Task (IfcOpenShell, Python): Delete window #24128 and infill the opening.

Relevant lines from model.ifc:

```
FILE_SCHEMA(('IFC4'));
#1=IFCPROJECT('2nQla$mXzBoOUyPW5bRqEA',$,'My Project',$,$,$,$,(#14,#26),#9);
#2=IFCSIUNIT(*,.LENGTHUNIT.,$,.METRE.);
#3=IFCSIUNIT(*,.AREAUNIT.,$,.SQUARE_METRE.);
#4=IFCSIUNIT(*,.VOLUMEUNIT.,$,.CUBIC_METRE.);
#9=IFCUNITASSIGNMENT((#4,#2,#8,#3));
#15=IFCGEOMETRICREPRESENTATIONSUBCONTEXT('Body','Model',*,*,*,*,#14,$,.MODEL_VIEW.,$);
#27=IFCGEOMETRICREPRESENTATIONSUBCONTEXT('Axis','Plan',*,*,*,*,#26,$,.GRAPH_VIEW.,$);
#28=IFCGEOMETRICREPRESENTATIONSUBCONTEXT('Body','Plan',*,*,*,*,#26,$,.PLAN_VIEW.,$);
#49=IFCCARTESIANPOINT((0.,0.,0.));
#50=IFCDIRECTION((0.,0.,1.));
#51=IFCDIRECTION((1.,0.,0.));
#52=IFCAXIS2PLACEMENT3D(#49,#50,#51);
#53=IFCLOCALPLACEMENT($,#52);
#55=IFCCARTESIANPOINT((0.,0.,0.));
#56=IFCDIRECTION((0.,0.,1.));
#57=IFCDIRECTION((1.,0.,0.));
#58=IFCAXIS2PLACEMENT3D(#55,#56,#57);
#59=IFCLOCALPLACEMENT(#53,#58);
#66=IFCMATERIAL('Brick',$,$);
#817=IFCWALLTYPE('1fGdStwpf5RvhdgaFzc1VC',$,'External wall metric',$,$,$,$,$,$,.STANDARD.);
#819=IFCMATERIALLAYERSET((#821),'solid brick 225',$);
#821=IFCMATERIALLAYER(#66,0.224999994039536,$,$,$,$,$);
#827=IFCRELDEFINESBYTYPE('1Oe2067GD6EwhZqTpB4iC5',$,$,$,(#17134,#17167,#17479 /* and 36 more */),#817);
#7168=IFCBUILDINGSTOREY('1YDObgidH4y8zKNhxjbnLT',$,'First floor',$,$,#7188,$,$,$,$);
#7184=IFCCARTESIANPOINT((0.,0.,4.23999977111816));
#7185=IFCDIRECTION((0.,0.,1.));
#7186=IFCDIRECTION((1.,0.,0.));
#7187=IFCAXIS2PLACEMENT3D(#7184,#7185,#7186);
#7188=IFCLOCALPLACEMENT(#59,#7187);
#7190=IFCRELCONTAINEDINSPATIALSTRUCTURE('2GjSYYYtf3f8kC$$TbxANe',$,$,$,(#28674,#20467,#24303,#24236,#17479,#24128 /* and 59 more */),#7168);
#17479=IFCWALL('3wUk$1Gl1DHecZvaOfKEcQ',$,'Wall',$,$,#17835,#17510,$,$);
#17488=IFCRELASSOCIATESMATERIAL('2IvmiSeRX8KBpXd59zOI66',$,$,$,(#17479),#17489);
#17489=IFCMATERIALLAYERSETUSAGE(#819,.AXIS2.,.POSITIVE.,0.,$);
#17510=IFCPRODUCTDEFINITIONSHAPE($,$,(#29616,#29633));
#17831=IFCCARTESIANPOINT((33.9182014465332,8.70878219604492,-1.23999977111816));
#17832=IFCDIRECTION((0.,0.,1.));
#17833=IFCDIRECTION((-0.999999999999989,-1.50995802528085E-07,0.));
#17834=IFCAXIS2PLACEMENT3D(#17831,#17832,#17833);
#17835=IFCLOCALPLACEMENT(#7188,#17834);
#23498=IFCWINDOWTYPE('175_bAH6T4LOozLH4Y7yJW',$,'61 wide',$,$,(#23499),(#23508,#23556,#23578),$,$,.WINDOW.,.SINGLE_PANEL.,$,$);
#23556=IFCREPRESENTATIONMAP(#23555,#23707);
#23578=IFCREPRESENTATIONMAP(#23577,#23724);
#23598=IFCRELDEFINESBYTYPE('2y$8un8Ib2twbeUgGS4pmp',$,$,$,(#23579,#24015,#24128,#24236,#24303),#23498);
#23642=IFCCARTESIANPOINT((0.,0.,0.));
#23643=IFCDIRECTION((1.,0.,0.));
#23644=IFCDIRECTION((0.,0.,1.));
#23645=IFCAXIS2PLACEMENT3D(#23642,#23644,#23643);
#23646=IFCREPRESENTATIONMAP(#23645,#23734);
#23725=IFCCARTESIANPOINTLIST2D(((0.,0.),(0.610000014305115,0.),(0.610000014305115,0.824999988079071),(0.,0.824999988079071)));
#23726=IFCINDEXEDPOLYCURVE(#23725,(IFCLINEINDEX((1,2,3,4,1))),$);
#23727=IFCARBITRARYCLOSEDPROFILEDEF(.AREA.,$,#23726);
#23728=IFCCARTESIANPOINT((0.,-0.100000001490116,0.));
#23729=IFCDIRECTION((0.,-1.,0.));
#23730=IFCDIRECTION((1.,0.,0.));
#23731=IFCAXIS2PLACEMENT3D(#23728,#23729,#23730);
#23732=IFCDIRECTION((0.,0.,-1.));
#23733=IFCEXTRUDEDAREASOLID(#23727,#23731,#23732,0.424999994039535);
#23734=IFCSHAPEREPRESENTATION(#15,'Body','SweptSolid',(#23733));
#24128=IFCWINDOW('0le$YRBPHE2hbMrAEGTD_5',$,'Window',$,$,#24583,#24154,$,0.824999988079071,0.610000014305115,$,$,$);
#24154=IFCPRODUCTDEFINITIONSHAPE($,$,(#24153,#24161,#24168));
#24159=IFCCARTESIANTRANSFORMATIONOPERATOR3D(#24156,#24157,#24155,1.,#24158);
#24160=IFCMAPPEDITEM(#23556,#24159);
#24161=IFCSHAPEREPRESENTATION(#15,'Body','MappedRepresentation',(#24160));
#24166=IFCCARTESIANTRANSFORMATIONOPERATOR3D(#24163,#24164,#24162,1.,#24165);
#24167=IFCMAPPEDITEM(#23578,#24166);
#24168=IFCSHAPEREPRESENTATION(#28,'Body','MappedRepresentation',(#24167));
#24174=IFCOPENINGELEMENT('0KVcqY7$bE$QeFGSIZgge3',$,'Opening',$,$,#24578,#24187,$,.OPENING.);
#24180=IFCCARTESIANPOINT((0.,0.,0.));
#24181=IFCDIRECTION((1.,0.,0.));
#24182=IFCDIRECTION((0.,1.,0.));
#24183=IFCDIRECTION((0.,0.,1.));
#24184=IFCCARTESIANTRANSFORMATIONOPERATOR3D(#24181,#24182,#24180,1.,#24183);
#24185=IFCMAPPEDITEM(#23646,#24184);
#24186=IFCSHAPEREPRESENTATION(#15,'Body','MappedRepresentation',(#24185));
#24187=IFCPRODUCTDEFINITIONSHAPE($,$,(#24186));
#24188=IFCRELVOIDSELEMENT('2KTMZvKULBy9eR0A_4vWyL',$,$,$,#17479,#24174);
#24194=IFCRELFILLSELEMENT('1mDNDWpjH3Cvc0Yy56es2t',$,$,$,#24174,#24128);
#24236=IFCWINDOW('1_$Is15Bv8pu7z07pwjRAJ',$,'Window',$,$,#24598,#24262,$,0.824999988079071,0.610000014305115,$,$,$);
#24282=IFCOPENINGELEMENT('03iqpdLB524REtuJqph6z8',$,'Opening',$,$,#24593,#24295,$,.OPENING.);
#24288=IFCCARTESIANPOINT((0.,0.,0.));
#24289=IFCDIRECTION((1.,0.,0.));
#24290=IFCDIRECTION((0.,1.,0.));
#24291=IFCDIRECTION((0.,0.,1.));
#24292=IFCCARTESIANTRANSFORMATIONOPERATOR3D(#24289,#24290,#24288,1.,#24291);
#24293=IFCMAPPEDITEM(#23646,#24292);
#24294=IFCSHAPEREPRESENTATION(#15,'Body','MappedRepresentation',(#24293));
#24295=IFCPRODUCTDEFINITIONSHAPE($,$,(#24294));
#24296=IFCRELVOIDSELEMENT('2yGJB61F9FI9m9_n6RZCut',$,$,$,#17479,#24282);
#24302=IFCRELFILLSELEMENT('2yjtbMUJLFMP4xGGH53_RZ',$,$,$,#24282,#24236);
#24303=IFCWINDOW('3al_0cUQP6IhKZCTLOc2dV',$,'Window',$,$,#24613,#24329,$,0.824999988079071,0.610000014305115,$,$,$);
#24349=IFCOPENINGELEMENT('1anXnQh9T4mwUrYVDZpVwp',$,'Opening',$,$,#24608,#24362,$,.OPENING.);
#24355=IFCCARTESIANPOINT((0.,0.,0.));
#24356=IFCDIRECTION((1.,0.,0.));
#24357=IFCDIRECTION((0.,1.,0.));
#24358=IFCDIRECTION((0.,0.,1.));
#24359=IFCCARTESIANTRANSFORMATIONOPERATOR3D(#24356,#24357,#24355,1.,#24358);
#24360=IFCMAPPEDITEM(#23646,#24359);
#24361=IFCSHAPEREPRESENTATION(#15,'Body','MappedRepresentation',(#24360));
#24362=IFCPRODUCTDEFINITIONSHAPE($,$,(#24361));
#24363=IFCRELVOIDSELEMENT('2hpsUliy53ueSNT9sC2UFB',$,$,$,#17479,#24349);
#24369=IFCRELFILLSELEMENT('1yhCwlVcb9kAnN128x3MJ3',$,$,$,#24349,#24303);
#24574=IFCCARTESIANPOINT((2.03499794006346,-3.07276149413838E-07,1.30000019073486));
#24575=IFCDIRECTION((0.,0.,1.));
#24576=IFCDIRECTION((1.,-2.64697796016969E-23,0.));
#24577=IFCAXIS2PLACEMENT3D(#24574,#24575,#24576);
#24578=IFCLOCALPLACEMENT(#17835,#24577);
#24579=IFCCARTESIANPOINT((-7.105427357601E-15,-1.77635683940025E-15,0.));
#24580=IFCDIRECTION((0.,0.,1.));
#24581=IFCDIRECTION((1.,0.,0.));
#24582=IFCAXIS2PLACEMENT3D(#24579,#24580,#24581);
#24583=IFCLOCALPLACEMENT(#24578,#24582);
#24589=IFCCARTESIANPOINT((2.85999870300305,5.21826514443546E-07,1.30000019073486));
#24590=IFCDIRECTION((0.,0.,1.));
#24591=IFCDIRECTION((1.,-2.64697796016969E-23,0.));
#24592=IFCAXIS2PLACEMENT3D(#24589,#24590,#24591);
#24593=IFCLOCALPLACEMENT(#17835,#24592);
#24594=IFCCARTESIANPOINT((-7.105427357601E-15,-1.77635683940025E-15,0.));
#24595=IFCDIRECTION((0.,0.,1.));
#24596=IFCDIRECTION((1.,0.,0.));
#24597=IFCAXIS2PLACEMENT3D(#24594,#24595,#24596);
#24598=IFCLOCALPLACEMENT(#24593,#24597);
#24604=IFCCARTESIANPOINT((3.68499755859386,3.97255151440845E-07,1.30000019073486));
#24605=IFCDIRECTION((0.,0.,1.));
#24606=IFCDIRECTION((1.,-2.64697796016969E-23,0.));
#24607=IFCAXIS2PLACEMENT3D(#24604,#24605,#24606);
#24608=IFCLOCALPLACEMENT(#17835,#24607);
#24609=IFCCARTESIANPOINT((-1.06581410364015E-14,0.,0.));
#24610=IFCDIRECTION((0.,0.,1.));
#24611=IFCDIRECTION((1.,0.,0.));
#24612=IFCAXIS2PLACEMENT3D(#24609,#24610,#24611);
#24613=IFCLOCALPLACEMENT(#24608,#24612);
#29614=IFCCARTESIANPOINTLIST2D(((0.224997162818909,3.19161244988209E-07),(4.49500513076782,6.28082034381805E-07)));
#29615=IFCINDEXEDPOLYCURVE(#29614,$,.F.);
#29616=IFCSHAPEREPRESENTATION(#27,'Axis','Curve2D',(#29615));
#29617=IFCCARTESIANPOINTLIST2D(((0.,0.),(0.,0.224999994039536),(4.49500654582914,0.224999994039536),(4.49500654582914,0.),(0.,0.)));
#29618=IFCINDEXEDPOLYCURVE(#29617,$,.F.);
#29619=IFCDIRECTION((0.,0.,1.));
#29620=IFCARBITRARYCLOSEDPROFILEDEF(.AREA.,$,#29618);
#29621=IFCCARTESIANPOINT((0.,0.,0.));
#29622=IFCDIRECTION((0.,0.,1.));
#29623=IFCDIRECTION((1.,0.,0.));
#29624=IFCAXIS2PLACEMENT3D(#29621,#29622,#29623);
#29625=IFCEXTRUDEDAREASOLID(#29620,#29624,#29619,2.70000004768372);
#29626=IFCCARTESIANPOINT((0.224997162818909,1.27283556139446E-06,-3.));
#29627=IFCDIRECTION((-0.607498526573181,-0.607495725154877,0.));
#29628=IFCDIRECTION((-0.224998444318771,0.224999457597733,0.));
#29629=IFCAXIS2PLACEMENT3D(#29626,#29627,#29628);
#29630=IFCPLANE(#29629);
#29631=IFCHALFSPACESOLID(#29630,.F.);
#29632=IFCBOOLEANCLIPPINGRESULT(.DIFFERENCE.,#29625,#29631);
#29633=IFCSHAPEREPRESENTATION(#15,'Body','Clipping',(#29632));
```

```python
import ifcopenshell
import ifcopenshell.api.feature
import ifcopenshell.api.root
import ifcopenshell.geom
import ifcopenshell.util.shape

model = ifcopenshell.open("model.ifc")
settings = ifcopenshell.geom.settings()


def volume(element):
    """Net volume in cubic metres, openings subtracted."""
    shape = ifcopenshell.geom.create_shape(settings, element)
    return ifcopenshell.util.shape.get_volume(shape.geometry)


window = model.by_id(24128)
opening = window.FillsVoids[0].RelatingOpeningElement
wall = opening.VoidsElements[0].RelatingBuildingElement
before = volume(wall)

ifcopenshell.api.root.remove_product(model, product=window)
ifcopenshell.api.feature.remove_feature(model, feature=opening)

after = volume(wall)

print(f"wall volume {before:.3f} -> {after:.3f} m3")

model.write("model-out.ifc")
```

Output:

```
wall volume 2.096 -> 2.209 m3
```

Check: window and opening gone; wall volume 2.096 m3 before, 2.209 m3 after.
